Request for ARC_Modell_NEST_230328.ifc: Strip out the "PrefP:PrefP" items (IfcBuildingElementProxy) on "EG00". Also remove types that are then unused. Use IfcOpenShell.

First a look at what the model holds.

```python
import ifcopenshell
import ifcopenshell.util.element

model = ifcopenshell.open("ARC_Modell_NEST_230328.ifc")
print(model.schema)
storey = next(s for s in model.by_type("IfcBuildingStorey") if s.Name == "EG00")
proxies = [e for e in ifcopenshell.util.element.get_decomposition(storey) if e.is_a("IfcBuildingElementProxy")]
seen = {}
for e in proxies:
    element_type = ifcopenshell.util.element.get_type(e)
    name = element_type.Name if element_type not in (None, e) else None
    seen[name] = seen.get(name, 0) + 1
for name, count in sorted(seen.items(), key=str):
    print(count, "x", name)
```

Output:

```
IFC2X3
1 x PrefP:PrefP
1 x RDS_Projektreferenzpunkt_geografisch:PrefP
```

```python
import ifcopenshell
import ifcopenshell.api.root
import ifcopenshell.util.element

model = ifcopenshell.open("ARC_Modell_NEST_230328.ifc")

storey = next(s for s in model.by_type("IfcBuildingStorey") if s.Name == "EG00")
proxies = [e for e in ifcopenshell.util.element.get_decomposition(storey) if e.is_a("IfcBuildingElementProxy")]
targets = [e for e in proxies if (t := ifcopenshell.util.element.get_type(e)) not in (None, e) and t.Name == "PrefP:PrefP"]
types = {ifcopenshell.util.element.get_type(e) for e in targets} - {None, *targets}

for e in targets:
    ifcopenshell.api.root.remove_product(model, product=e)
print(len(targets), "removed")

unused = [t for t in types if not ifcopenshell.util.element.get_types(t)]
for t in unused:
    ifcopenshell.api.root.remove_product(model, product=t)
print(len(unused), "unused types removed")

model.write("ARC_Modell_NEST_230328_rev.ifc")
```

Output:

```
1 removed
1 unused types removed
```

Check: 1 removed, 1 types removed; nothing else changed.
